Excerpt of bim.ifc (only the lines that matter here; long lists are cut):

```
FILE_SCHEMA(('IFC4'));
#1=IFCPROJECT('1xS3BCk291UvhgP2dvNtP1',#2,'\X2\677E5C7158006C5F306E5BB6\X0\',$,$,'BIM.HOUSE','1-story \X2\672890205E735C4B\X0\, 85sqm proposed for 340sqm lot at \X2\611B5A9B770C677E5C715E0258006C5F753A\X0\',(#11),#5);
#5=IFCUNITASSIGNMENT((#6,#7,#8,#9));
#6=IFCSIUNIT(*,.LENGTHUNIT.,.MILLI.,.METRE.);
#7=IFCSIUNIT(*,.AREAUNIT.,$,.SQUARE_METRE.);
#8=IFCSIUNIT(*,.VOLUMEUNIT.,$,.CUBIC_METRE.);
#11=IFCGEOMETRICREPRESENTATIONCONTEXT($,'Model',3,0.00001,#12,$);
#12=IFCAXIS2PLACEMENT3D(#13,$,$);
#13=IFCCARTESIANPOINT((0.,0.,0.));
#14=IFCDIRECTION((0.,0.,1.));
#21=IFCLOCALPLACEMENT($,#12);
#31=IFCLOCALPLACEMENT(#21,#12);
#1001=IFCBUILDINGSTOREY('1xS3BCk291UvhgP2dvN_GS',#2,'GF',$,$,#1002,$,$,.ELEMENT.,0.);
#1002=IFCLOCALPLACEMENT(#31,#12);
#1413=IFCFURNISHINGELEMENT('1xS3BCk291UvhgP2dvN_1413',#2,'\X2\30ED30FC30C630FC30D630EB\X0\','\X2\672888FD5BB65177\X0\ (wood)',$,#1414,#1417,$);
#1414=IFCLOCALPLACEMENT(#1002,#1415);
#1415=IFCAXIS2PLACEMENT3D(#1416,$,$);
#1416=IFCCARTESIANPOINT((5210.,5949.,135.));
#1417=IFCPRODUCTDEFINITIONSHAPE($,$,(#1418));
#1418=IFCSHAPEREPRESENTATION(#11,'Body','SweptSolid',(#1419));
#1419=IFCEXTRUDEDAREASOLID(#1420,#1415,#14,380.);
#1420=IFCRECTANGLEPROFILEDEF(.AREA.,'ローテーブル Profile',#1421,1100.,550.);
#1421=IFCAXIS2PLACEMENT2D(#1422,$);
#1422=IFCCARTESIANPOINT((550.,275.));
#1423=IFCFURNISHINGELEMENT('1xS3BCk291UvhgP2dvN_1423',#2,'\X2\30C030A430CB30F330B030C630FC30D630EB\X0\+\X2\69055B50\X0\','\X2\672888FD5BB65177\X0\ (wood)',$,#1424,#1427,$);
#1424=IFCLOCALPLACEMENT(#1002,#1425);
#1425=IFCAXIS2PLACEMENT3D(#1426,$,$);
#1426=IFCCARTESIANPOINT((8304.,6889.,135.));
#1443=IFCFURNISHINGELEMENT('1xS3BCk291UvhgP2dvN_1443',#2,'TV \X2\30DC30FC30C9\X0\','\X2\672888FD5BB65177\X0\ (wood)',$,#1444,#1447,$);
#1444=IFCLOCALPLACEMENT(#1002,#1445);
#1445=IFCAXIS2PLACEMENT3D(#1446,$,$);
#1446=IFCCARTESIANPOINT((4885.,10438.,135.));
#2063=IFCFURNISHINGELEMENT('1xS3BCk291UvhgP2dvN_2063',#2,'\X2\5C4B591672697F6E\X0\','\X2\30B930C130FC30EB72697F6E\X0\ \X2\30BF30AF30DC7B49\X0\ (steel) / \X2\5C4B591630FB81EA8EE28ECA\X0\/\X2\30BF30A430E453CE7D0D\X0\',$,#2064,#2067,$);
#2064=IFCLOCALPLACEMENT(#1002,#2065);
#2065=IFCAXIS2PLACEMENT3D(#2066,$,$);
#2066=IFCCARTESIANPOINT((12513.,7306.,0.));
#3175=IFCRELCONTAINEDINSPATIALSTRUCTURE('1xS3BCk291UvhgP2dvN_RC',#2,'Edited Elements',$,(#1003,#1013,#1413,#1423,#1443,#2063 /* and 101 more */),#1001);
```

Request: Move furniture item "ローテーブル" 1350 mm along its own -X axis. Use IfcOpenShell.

```python
import ifcopenshell
import ifcopenshell.api.geometry
import ifcopenshell.util.placement
import ifcopenshell.util.unit

model = ifcopenshell.open("bim.ifc")
unit_scale = ifcopenshell.util.unit.calculate_unit_scale(model)

item = model.by_guid("1xS3BCk291UvhgP2dvN_1413")
matrix = ifcopenshell.util.placement.get_local_placement(item.ObjectPlacement)
matrix[:3, 3] -= matrix[:3, 0] * 1.35 / unit_scale
ifcopenshell.api.geometry.edit_object_placement(model, product=item, matrix=matrix, is_si=False)

print(ifcopenshell.util.placement.get_local_placement(item.ObjectPlacement).round(3) + 0.0)

model.write("bim_v2.ifc")
```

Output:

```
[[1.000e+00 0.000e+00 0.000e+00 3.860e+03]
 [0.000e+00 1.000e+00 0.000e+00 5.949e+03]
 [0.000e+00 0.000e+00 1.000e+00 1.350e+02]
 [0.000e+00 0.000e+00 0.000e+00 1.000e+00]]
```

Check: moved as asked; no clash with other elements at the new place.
